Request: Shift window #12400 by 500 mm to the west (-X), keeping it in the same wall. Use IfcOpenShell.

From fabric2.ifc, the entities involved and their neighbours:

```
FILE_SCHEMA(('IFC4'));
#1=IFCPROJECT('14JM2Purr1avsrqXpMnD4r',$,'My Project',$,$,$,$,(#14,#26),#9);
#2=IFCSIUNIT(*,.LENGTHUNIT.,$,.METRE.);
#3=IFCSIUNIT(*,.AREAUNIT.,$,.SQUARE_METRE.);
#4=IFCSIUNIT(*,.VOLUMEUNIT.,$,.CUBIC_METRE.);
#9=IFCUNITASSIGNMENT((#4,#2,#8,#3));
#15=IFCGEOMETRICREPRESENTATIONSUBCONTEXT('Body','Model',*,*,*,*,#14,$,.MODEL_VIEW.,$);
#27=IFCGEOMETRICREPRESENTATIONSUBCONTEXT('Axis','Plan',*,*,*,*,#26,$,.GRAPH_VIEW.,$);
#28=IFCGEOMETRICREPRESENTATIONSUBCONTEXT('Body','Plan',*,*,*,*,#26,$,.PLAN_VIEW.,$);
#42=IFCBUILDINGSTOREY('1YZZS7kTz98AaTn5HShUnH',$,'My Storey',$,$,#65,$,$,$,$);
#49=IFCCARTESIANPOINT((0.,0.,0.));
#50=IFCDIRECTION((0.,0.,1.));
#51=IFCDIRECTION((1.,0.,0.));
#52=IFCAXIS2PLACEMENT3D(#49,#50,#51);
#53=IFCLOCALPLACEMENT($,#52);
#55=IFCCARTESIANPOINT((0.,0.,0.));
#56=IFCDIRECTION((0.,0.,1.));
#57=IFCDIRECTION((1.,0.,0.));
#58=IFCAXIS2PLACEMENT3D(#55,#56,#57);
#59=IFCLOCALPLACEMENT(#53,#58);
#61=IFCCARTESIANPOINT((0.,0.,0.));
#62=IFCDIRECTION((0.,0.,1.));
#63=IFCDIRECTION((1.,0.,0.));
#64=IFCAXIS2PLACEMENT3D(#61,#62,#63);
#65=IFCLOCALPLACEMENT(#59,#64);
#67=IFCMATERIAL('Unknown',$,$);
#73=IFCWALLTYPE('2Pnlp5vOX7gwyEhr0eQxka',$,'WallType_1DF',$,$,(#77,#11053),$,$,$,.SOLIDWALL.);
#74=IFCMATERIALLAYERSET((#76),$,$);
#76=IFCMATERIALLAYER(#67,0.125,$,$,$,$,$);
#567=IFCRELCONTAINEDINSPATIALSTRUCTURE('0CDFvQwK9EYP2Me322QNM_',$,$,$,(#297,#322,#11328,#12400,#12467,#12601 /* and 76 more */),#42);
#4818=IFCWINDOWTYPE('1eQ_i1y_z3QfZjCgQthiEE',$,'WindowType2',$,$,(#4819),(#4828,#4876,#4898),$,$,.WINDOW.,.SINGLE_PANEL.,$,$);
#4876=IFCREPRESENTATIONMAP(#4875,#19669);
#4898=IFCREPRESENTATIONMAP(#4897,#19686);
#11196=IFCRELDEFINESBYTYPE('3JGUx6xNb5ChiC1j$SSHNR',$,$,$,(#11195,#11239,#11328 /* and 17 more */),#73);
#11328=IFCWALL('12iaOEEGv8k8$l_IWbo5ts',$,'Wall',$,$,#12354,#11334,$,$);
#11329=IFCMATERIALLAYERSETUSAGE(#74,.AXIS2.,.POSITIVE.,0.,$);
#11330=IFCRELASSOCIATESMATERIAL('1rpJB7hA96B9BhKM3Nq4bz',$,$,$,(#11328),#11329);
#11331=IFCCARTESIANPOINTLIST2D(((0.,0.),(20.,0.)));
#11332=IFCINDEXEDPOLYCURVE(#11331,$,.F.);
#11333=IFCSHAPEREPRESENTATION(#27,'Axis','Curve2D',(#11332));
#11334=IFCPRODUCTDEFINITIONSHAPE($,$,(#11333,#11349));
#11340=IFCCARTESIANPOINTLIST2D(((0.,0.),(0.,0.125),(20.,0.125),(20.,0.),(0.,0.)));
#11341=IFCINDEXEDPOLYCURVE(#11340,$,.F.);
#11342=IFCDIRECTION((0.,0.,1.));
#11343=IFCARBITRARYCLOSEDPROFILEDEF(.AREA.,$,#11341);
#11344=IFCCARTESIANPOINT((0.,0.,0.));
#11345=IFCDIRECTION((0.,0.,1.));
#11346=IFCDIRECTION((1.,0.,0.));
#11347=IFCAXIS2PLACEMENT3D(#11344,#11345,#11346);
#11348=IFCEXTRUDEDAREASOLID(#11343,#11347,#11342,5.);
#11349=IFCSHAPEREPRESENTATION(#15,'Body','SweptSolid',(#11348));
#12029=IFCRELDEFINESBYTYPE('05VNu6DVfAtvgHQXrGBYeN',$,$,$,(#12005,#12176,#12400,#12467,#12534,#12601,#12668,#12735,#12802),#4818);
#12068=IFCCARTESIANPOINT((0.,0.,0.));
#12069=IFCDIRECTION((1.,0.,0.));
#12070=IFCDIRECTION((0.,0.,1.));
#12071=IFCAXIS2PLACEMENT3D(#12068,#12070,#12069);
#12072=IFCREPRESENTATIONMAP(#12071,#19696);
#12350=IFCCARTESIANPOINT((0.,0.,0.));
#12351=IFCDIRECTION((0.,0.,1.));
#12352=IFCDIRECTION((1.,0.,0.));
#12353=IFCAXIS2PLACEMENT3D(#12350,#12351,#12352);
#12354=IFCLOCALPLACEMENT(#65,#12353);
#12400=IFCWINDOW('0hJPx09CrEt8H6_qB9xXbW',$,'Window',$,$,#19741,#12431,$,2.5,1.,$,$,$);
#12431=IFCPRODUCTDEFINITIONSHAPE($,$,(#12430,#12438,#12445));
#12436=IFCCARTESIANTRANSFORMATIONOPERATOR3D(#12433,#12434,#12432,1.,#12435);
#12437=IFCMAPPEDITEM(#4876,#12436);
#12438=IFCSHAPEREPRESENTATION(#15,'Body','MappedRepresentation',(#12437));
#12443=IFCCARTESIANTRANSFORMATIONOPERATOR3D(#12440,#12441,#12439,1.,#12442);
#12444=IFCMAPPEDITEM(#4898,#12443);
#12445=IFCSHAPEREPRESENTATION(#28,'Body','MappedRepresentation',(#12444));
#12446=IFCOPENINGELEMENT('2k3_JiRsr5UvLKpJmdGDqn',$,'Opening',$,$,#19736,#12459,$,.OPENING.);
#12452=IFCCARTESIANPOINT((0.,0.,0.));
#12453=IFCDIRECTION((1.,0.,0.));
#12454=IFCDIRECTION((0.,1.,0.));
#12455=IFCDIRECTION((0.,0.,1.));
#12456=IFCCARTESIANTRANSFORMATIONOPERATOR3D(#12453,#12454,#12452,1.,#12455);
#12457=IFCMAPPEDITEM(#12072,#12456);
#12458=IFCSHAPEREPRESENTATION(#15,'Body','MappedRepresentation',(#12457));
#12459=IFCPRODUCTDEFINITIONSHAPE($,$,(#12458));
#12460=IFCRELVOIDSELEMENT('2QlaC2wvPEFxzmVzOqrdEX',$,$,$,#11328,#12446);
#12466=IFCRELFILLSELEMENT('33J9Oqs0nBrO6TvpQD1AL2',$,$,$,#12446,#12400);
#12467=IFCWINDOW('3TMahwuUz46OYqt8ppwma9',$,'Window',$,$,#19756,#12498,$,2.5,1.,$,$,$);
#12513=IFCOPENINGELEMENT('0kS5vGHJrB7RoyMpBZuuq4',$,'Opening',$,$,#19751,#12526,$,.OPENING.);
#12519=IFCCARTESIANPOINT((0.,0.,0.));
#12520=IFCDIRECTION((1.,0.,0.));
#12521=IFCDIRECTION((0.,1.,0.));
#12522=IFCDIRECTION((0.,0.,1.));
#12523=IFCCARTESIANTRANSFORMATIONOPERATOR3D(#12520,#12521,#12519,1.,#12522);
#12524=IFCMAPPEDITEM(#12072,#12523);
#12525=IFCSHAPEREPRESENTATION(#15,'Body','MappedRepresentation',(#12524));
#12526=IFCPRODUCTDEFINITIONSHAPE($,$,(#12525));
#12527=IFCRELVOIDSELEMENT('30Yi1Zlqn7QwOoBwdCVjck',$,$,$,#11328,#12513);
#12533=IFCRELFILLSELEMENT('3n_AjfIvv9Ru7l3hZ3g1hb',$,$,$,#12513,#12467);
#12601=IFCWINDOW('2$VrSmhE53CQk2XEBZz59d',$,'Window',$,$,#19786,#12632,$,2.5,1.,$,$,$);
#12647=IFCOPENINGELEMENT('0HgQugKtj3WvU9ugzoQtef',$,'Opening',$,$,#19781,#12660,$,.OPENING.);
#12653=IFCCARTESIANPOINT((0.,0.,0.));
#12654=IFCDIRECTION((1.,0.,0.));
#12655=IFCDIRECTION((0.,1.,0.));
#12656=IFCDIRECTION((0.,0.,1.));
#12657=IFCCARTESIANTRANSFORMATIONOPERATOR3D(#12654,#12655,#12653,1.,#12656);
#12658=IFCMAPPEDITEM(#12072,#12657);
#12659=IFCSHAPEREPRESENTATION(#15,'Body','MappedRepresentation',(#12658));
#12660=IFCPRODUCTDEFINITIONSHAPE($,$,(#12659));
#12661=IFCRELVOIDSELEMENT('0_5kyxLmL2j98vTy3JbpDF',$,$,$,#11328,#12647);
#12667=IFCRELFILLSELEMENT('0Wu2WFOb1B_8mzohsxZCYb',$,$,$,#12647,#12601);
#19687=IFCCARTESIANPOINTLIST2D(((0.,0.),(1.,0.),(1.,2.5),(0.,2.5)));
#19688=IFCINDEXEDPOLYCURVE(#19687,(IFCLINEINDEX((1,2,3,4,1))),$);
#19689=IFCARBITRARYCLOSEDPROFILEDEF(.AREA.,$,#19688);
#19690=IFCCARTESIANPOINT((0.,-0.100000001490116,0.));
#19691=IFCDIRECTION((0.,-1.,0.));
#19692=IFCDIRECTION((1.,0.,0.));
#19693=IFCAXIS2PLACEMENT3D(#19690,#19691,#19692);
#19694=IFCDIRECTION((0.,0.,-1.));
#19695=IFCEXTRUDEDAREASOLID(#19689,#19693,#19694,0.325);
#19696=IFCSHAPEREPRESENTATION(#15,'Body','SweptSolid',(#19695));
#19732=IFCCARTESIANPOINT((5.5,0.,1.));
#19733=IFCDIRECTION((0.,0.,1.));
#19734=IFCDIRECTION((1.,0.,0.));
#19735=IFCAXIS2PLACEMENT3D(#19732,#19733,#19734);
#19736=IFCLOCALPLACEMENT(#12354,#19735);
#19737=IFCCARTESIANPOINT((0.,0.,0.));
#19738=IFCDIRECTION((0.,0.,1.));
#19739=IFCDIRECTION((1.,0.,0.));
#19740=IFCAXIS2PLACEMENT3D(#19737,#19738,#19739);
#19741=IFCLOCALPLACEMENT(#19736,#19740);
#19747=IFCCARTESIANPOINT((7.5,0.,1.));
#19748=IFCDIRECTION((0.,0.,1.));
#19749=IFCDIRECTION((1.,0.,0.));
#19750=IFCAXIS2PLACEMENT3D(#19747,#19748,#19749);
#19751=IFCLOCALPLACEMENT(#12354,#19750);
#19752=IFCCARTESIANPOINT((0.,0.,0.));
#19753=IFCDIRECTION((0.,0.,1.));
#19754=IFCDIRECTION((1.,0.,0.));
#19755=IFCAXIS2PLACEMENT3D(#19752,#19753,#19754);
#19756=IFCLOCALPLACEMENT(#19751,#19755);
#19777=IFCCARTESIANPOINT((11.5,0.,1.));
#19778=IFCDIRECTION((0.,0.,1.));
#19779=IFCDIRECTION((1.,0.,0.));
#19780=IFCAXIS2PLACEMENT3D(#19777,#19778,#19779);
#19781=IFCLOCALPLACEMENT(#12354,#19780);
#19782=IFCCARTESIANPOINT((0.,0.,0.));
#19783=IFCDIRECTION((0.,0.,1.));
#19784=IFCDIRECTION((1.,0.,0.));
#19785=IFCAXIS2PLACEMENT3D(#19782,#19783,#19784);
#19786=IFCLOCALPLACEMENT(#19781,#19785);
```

```python
import ifcopenshell
import ifcopenshell.api.geometry
import ifcopenshell.util.placement
import ifcopenshell.util.unit

model = ifcopenshell.open("fabric2.ifc")
unit_scale = ifcopenshell.util.unit.calculate_unit_scale(model)

window = model.by_id(12400)
opening = window.FillsVoids[0].RelatingOpeningElement
wall = opening.VoidsElements[0].RelatingBuildingElement

wall_matrix = ifcopenshell.util.placement.get_local_placement(wall.ObjectPlacement)
shift = wall_matrix[:3, 0] * -0.5 / unit_scale
before = ifcopenshell.util.placement.get_local_placement(window.ObjectPlacement)[:3, 3].copy()

# The window is placed relative to its opening, so it follows when the opening moves.
matrix = ifcopenshell.util.placement.get_local_placement(opening.ObjectPlacement)
matrix[:3, 3] += shift
ifcopenshell.api.geometry.edit_object_placement(
    model, product=opening, matrix=matrix, is_si=False, should_transform_children=True
)

after = ifcopenshell.util.placement.get_local_placement(window.ObjectPlacement)[:3, 3]
print("window moved by", (after - before).round(3) + 0.0)

model.write("fabric2-out.ifc")
```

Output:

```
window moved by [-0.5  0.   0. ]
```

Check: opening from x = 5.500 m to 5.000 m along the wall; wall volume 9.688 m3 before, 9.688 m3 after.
